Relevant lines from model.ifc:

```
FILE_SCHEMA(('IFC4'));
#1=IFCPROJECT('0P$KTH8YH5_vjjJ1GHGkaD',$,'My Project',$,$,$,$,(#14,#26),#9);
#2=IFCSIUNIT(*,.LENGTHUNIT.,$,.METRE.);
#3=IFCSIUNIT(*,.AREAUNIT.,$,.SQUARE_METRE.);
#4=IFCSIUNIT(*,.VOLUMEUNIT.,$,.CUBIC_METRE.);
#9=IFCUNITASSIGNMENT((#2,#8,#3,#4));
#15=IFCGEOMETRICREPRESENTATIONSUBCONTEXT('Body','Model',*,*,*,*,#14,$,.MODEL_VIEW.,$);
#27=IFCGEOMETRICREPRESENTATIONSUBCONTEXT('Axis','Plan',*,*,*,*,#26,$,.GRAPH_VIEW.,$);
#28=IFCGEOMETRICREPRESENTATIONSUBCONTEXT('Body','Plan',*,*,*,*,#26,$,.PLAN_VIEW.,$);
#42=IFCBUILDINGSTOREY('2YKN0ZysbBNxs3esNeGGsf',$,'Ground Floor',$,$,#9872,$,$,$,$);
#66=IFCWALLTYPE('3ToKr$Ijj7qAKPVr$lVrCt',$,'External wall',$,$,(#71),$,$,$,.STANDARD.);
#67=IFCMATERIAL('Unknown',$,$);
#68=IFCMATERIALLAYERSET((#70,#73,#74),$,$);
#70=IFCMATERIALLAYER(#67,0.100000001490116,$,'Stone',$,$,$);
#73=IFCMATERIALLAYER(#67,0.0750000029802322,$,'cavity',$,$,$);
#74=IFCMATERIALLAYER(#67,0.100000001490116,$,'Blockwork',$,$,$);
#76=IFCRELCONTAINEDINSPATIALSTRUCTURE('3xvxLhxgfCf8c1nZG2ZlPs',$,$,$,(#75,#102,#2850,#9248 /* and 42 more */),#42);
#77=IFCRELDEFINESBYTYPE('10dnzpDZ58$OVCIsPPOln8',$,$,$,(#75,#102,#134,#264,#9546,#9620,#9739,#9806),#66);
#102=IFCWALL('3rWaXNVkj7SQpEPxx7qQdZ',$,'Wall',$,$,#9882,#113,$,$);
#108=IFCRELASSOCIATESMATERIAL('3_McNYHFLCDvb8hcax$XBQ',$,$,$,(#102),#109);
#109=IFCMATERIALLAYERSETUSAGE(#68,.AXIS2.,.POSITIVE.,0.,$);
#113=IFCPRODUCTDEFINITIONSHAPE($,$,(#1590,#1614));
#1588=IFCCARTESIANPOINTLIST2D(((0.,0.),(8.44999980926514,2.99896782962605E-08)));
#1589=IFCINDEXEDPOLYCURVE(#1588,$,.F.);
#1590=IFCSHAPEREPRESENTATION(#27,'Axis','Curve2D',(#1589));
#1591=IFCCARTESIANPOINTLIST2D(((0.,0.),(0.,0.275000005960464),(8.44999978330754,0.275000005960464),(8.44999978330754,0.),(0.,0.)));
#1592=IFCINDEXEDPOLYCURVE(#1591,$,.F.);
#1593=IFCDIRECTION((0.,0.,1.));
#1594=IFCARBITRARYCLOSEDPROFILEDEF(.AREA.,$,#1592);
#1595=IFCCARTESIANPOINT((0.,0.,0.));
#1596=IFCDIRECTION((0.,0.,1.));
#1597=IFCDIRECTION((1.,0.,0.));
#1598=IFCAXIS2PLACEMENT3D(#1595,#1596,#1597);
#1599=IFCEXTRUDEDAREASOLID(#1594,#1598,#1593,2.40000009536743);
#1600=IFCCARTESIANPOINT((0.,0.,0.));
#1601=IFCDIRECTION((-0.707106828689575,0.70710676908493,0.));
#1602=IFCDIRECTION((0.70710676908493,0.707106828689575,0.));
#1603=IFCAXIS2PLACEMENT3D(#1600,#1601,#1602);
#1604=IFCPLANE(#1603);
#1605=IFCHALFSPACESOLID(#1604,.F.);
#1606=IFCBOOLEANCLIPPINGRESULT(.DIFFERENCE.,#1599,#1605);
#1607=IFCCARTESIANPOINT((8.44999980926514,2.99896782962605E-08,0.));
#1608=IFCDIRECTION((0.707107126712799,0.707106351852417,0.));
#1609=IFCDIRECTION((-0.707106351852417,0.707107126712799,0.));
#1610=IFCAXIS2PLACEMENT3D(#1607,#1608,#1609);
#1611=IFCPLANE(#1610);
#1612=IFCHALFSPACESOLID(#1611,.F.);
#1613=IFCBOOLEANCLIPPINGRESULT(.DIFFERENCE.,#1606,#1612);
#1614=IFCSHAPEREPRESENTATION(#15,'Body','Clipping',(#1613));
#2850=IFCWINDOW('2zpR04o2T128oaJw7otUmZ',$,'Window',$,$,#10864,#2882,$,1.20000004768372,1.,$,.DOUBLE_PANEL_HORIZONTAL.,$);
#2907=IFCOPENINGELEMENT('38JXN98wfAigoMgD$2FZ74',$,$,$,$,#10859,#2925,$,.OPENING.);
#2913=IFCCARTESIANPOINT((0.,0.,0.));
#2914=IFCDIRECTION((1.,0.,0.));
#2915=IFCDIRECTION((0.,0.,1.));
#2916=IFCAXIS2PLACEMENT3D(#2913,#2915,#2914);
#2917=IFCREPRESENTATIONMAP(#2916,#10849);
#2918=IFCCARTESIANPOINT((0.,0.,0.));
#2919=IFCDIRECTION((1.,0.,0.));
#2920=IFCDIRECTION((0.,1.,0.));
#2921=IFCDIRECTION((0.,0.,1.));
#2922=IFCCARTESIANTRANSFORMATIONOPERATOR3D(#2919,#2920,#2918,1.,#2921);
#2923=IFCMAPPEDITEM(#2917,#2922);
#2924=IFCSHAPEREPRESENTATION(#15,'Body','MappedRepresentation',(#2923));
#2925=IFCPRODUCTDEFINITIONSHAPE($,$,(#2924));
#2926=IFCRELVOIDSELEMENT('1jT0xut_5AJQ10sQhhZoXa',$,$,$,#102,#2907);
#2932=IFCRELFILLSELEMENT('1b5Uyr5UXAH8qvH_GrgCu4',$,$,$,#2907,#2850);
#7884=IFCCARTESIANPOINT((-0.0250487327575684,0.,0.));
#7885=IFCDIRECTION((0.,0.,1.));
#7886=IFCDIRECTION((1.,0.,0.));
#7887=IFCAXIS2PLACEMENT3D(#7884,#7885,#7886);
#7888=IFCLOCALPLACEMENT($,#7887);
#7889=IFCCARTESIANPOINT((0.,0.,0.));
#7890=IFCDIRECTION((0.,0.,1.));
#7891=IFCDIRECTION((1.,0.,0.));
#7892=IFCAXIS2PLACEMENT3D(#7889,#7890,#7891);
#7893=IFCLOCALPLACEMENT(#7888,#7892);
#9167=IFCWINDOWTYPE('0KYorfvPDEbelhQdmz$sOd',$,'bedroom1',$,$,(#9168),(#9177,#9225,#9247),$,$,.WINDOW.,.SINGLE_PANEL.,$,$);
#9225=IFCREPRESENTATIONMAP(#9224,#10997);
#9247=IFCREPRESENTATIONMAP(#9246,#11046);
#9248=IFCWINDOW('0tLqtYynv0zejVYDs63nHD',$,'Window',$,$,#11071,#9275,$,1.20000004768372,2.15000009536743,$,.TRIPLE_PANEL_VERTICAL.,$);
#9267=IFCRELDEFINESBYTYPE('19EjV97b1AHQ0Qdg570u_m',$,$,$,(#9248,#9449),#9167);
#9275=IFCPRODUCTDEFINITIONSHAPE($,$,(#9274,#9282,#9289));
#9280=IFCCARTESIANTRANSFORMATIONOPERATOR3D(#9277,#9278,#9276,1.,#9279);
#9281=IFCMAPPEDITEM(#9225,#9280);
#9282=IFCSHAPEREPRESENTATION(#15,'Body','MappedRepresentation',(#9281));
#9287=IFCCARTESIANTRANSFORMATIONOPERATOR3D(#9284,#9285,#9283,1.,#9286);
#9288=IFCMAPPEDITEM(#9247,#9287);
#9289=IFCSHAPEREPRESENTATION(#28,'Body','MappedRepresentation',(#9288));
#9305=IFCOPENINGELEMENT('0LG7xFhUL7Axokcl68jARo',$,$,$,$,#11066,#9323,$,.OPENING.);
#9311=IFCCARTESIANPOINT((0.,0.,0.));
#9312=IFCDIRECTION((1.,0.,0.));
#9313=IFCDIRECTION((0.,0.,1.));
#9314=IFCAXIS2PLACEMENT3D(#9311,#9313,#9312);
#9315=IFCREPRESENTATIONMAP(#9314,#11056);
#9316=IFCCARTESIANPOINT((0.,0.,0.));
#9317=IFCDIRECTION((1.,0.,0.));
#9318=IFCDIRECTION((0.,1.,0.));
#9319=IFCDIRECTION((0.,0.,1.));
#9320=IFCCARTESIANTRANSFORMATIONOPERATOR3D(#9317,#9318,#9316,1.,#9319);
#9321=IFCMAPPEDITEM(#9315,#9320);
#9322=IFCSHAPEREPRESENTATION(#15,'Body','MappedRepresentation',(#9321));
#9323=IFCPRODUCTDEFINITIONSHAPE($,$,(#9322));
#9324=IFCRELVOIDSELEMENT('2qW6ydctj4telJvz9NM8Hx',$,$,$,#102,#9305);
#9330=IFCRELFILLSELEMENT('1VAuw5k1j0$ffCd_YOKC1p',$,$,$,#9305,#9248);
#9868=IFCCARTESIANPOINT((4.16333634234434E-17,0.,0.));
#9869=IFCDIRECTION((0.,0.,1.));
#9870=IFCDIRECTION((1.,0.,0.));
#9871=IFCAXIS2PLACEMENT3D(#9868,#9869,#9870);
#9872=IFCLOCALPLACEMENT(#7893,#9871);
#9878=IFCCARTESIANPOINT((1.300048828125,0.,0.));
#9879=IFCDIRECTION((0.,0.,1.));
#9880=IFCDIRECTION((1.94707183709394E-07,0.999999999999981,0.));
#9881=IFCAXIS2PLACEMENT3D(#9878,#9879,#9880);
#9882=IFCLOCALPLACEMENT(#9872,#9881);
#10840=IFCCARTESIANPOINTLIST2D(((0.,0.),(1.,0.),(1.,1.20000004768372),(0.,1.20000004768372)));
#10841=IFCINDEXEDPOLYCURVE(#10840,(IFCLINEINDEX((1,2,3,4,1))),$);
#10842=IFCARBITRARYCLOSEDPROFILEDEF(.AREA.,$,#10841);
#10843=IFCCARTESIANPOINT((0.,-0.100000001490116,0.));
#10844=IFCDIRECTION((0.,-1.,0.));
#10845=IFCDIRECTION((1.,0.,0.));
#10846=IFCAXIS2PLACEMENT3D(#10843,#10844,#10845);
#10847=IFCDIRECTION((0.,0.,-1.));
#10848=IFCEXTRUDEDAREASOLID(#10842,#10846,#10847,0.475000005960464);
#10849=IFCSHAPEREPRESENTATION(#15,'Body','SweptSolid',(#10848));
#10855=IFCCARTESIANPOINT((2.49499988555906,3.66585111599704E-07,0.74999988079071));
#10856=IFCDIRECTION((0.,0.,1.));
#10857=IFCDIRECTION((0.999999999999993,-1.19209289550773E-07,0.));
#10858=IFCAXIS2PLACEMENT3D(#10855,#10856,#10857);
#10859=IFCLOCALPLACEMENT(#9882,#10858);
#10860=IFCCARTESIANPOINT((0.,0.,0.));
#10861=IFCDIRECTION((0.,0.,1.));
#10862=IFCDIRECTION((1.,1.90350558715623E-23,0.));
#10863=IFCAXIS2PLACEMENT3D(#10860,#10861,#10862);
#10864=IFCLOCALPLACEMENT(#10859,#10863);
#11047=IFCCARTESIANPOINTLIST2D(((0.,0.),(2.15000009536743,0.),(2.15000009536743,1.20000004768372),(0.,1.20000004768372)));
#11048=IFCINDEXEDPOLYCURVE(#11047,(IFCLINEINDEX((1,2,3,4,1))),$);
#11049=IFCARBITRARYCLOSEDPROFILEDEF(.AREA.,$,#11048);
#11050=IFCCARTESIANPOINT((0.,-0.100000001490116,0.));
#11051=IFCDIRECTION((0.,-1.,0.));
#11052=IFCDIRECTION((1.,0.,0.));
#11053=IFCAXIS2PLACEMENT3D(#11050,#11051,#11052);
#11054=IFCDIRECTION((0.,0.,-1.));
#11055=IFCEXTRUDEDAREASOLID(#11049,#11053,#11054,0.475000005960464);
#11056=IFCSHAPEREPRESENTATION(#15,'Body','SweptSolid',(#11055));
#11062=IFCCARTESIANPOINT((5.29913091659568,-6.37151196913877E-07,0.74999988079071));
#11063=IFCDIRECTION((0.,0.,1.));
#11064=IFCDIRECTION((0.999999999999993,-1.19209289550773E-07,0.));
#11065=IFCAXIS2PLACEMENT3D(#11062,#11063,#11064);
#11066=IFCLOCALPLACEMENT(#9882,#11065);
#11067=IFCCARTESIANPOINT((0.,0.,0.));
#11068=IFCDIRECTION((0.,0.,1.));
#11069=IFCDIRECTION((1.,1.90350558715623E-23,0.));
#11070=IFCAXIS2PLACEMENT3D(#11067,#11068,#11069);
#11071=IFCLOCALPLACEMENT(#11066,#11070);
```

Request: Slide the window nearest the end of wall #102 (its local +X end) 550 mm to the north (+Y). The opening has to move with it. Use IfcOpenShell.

```python
import ifcopenshell
import ifcopenshell.api.geometry
import ifcopenshell.util.placement
import ifcopenshell.util.unit

model = ifcopenshell.open("model.ifc")
unit_scale = ifcopenshell.util.unit.calculate_unit_scale(model)

window = model.by_id(9248)
opening = window.FillsVoids[0].RelatingOpeningElement
wall = opening.VoidsElements[0].RelatingBuildingElement

wall_matrix = ifcopenshell.util.placement.get_local_placement(wall.ObjectPlacement)
shift = wall_matrix[:3, 0] * 0.55 / unit_scale
before = ifcopenshell.util.placement.get_local_placement(window.ObjectPlacement)[:3, 3].copy()

# The window is placed relative to its opening, so it follows when the opening moves.
matrix = ifcopenshell.util.placement.get_local_placement(opening.ObjectPlacement)
matrix[:3, 3] += shift
ifcopenshell.api.geometry.edit_object_placement(
    model, product=opening, matrix=matrix, is_si=False, should_transform_children=True
)

after = ifcopenshell.util.placement.get_local_placement(window.ObjectPlacement)[:3, 3]
print("window moved by", (after - before).round(3) + 0.0)

model.write("model_updated.ifc")
```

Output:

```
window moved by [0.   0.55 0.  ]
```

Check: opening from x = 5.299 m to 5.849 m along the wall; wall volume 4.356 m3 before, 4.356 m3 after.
